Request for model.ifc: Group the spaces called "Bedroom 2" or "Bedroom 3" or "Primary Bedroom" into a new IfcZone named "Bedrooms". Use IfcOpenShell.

First a look at what the model holds.

```python
import ifcopenshell

model = ifcopenshell.open("model.ifc")
print(model.schema)
seen = {}
for space in model.by_type("IfcSpace"):
    seen[space.LongName] = seen.get(space.LongName, 0) + 1
for name, count in sorted(seen.items(), key=str):
    print(count, "x", name)
print("zones:", [z.Name for z in model.by_type("IfcZone")][:20])
```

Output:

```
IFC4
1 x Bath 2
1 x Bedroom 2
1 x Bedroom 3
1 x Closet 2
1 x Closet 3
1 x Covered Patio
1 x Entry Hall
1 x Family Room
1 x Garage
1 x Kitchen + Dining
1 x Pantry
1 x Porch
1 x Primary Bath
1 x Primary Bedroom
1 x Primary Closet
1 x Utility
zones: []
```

```python
import ifcopenshell
import ifcopenshell.api.group
import ifcopenshell.api.root

model = ifcopenshell.open("model.ifc")

names = {"Bedroom 2", "Bedroom 3", "Primary Bedroom"}
spaces = [s for s in model.by_type("IfcSpace") if s.LongName in names]

zone = ifcopenshell.api.root.create_entity(model, ifc_class="IfcZone", name="Bedrooms")
ifcopenshell.api.group.assign_group(model, products=spaces, group=zone)
print(len(spaces), "spaces in", zone.Name)

model.write("model-out.ifc")
```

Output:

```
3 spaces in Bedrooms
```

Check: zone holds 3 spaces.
